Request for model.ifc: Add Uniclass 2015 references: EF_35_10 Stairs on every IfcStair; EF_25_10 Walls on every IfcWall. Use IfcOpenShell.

First a look at what the model holds.

```python
import ifcopenshell

model = ifcopenshell.open("model.ifc")
print(model.schema)
print("classifications:", [c.Name for c in model.by_type("IfcClassification")])
for ifc_class in ("IfcDoor", "IfcRoof", "IfcStair", "IfcWall", "IfcWindow"):
    print(ifc_class, len(model.by_type(ifc_class)))
```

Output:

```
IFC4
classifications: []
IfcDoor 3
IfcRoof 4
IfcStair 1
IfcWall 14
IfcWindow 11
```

```python
import ifcopenshell
import ifcopenshell.api.classification

model = ifcopenshell.open("model.ifc")

system = ifcopenshell.api.classification.add_classification(model, classification="Uniclass 2015")

codes = {
    "IfcStair": ("EF_35_10", "Stairs"),
    "IfcWall": ("EF_25_10", "Walls"),
}
for ifc_class, (code, name) in codes.items():
    products = model.by_type(ifc_class)
    ifcopenshell.api.classification.add_reference(
        model, products=products, classification=system, identification=code, name=name
    )
    print(code, len(products))

model.write("model_updated.ifc")
```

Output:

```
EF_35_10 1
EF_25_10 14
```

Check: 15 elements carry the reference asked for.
